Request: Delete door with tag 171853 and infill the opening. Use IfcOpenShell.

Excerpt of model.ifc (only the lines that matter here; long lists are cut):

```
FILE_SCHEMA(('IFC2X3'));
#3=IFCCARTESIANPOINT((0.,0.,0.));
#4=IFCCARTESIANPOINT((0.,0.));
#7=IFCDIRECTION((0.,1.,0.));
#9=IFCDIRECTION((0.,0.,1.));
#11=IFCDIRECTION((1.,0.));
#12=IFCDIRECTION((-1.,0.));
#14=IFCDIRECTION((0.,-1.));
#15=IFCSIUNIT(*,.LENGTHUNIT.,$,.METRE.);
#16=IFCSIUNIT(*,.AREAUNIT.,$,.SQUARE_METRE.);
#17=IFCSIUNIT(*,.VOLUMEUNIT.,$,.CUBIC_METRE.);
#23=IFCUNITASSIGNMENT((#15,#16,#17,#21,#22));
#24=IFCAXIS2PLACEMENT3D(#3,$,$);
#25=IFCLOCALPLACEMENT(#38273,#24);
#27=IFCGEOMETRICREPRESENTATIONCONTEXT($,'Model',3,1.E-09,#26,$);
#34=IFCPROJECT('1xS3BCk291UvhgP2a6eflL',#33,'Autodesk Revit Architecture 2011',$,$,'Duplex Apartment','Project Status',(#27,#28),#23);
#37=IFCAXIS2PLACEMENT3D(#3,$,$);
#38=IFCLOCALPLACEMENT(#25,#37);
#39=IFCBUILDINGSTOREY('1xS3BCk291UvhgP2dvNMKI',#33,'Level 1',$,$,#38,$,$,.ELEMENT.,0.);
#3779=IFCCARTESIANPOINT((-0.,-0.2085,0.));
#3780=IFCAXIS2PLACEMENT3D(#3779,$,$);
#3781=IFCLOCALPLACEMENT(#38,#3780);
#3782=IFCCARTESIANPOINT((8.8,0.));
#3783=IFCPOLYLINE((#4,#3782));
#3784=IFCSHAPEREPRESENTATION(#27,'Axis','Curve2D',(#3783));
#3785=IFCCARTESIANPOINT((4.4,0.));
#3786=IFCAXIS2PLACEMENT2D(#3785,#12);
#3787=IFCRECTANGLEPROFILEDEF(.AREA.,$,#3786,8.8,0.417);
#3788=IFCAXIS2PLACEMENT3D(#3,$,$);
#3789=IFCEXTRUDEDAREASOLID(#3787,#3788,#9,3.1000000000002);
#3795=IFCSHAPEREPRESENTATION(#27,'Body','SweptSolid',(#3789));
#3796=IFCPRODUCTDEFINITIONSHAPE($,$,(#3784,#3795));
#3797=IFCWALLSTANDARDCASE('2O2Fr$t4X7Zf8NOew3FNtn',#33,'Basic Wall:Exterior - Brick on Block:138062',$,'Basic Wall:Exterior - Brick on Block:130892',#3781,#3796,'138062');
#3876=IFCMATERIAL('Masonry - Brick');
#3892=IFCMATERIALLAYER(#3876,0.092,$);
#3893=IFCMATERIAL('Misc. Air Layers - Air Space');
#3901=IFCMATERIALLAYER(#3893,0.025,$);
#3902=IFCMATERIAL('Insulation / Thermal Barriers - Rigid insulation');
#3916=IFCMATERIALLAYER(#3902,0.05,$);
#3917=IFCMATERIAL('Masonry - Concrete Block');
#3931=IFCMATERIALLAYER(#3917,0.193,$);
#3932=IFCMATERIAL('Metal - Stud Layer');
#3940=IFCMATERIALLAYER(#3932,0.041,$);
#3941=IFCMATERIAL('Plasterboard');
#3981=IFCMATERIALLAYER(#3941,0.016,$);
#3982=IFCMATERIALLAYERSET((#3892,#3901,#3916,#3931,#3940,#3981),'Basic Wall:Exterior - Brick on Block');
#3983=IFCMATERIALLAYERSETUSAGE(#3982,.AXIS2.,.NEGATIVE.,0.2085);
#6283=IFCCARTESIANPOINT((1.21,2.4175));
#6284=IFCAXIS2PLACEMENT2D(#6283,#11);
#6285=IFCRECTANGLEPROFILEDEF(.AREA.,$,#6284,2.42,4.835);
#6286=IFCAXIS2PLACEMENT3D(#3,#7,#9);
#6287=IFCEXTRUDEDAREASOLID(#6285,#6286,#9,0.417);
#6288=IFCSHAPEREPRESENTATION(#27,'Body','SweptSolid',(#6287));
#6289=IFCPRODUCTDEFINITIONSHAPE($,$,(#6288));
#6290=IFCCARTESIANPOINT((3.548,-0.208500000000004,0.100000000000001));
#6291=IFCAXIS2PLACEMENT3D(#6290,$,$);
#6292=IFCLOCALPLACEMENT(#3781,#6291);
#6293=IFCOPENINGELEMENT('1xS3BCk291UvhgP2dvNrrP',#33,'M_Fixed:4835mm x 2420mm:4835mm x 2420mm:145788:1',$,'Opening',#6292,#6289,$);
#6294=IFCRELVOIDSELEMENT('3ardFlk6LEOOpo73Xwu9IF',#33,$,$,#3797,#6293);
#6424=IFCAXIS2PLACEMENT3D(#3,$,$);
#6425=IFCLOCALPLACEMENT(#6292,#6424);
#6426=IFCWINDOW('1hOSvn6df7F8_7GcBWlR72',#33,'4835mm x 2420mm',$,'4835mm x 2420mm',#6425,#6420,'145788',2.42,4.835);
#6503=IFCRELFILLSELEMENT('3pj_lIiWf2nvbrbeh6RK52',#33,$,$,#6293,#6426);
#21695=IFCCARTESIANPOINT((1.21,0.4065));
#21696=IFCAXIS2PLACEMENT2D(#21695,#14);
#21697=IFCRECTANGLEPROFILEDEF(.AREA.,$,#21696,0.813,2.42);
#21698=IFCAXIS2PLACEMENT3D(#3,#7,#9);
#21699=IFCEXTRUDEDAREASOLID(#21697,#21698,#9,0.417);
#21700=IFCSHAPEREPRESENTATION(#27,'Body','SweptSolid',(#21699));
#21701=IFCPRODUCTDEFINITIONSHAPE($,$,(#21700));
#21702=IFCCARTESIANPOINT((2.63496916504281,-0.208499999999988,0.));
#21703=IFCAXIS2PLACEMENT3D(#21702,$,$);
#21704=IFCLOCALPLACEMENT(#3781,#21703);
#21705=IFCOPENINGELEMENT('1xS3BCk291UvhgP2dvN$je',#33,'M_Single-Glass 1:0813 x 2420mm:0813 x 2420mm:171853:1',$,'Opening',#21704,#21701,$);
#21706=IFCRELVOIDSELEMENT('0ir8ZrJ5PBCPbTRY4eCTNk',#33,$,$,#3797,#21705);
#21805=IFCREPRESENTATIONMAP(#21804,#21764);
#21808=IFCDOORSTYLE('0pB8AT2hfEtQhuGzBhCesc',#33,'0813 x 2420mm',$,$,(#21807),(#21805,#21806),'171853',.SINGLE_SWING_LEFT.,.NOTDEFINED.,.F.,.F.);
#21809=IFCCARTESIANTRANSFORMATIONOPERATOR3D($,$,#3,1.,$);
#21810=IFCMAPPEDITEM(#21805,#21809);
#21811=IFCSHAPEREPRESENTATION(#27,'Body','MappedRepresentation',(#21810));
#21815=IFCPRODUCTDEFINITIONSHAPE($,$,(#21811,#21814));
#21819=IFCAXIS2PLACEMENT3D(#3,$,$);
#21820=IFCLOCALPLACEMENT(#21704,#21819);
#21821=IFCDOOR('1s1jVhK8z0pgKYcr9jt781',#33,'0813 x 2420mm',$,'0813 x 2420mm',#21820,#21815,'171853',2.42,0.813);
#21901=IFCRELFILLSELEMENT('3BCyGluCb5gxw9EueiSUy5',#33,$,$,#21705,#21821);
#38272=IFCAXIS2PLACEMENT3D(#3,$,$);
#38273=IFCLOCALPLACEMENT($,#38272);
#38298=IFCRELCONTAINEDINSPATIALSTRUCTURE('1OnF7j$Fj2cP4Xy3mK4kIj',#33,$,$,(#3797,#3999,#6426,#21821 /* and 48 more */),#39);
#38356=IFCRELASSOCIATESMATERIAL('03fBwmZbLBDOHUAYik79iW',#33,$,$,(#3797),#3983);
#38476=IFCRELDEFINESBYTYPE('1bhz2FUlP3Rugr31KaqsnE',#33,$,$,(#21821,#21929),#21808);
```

```python
import ifcopenshell
import ifcopenshell.api.feature
import ifcopenshell.api.root
import ifcopenshell.geom
import ifcopenshell.util.shape

model = ifcopenshell.open("model.ifc")
settings = ifcopenshell.geom.settings()


def volume(element):
    """Net volume in cubic metres, openings subtracted."""
    shape = ifcopenshell.geom.create_shape(settings, element)
    return ifcopenshell.util.shape.get_volume(shape.geometry)


door = model.by_guid("1s1jVhK8z0pgKYcr9jt781")
opening = door.FillsVoids[0].RelatingOpeningElement
wall = opening.VoidsElements[0].RelatingBuildingElement
before = volume(wall)

ifcopenshell.api.root.remove_product(model, product=door)
ifcopenshell.api.feature.remove_feature(model, feature=opening)

after = volume(wall)

print(f"wall volume {before:.3f} -> {after:.3f} m3")

model.write("model_edited.ifc")
```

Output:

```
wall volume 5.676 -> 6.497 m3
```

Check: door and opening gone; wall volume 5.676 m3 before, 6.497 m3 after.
